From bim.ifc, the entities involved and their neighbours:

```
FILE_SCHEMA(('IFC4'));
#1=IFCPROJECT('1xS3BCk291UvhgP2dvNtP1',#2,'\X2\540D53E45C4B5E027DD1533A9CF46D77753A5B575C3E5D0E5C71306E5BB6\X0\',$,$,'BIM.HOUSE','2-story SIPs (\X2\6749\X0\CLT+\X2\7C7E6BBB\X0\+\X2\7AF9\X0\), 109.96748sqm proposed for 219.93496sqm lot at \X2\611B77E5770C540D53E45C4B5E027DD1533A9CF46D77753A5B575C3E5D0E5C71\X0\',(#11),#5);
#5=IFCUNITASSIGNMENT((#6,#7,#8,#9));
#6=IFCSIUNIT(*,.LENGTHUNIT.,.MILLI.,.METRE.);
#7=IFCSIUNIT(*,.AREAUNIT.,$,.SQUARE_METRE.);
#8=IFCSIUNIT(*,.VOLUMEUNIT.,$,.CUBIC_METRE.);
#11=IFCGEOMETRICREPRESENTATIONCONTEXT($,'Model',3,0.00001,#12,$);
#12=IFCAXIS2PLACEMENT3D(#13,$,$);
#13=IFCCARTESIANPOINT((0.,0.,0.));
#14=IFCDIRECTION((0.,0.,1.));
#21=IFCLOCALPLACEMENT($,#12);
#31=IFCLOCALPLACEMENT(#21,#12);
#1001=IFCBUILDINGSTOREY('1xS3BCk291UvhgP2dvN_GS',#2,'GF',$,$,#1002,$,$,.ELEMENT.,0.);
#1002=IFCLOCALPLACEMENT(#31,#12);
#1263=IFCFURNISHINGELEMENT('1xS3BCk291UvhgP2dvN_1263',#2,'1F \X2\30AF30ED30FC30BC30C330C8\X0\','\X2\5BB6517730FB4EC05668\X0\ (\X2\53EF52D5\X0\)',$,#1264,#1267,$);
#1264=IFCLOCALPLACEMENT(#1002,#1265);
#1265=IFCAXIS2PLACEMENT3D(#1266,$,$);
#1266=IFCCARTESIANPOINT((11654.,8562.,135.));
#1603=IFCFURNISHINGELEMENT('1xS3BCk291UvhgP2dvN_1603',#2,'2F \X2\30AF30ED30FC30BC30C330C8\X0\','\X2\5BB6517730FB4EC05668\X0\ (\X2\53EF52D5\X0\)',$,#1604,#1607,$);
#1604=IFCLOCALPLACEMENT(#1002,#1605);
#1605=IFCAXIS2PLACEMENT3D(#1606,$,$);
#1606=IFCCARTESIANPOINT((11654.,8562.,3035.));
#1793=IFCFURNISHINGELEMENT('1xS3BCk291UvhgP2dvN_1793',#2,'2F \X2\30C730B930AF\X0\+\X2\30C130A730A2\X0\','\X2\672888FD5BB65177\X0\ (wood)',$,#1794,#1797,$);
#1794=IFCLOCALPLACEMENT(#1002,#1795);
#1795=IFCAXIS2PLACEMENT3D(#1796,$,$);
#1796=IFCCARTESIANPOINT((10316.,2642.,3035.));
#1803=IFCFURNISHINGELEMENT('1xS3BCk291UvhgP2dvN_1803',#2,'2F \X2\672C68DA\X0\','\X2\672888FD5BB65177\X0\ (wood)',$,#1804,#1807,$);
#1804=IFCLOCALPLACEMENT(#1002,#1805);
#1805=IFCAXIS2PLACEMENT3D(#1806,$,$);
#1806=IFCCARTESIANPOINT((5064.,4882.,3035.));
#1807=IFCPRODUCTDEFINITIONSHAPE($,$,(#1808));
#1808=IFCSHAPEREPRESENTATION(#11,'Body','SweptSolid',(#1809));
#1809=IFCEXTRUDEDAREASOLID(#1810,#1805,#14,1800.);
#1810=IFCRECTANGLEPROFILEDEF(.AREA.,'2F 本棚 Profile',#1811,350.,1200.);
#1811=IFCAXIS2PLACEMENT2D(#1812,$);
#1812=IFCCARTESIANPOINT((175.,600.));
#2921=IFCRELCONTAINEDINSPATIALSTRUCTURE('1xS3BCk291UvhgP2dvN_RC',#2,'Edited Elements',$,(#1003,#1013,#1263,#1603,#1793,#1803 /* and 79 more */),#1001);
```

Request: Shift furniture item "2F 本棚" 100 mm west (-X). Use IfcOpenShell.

```python
import ifcopenshell
import ifcopenshell.api.geometry
import ifcopenshell.util.placement

model = ifcopenshell.open("bim.ifc")

item = model.by_id(1803)
matrix = ifcopenshell.util.placement.get_local_placement(item.ObjectPlacement)
matrix[0, 3] -= 100.0
ifcopenshell.api.geometry.edit_object_placement(model, product=item, matrix=matrix, is_si=False)

print(ifcopenshell.util.placement.get_local_placement(item.ObjectPlacement).round(3) + 0.0)

model.write("bim-out.ifc")
```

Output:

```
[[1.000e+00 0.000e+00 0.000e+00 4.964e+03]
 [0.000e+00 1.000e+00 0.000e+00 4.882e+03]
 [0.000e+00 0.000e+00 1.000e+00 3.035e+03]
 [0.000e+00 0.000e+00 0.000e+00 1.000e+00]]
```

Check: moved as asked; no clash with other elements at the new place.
